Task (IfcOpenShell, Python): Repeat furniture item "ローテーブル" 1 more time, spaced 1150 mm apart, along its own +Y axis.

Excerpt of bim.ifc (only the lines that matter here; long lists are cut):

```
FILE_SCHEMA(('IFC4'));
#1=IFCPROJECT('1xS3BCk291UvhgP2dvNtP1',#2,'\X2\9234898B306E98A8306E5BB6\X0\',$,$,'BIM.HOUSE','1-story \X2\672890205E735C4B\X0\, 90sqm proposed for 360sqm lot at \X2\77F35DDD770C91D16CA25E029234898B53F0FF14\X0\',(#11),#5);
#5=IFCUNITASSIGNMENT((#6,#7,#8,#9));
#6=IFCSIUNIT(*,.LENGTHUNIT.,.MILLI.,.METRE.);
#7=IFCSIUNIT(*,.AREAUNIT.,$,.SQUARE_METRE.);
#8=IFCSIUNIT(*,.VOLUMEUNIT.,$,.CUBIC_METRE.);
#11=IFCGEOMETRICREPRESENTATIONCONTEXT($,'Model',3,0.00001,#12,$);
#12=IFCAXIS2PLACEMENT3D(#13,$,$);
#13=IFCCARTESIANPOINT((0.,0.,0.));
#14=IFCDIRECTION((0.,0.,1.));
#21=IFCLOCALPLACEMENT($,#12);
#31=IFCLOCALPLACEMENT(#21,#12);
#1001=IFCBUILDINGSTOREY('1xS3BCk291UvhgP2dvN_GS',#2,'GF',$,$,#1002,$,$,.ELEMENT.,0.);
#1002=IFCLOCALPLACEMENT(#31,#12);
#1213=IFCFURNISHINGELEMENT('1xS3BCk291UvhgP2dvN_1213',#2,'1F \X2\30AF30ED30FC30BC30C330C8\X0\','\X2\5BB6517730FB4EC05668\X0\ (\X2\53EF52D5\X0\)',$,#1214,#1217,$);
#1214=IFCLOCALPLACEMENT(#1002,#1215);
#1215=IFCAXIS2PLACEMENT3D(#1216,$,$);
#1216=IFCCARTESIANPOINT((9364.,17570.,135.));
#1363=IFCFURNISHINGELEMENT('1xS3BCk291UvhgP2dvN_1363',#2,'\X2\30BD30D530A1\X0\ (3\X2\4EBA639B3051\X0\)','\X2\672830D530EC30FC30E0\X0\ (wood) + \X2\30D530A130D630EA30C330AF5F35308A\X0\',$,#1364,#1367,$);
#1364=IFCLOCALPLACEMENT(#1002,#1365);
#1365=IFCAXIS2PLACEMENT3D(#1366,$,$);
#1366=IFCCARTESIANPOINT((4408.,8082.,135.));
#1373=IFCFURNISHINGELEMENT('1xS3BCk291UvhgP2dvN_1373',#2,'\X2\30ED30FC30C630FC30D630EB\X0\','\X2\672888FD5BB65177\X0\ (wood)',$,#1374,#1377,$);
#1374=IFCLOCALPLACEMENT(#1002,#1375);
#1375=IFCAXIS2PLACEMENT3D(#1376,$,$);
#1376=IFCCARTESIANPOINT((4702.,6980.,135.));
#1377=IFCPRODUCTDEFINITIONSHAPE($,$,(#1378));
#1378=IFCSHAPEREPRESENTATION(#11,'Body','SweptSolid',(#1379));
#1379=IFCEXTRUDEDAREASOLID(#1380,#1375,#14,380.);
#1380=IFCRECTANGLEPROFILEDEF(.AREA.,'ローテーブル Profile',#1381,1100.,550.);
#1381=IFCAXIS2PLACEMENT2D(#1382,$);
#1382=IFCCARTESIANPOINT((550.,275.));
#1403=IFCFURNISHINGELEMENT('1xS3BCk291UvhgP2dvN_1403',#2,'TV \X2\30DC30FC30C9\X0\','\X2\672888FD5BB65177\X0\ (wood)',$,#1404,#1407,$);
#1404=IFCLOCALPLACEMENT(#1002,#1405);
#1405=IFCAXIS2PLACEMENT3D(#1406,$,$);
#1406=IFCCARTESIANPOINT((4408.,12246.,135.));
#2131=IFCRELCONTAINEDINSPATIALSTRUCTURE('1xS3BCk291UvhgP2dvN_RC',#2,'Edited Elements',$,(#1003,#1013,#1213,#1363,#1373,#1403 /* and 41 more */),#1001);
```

```python
import ifcopenshell
import ifcopenshell.api.geometry
import ifcopenshell.api.root
import ifcopenshell.util.element
import ifcopenshell.util.placement

model = ifcopenshell.open("bim.ifc")


def reuse_history(source, copy):
    """copy_class also copies each property set's owner history, people and application; keep the originals."""
    for rel in copy.IsDefinedBy:
        if rel.is_a("IfcRelDefinesByProperties") and (history := rel.RelatingPropertyDefinition.OwnerHistory):
            rel.RelatingPropertyDefinition.OwnerHistory = source.OwnerHistory
            ifcopenshell.util.element.remove_deep2(model, history)


source = model.by_id(1373)
base = ifcopenshell.util.placement.get_local_placement(source.ObjectPlacement)
step = base[:3, 1] * 1150.0

for i in range(1, 2):
    copy = ifcopenshell.api.root.copy_class(model, product=source)
    copy.Representation = ifcopenshell.util.element.copy_deep(
        model, source.Representation, exclude=["IfcGeometricRepresentationContext", "IfcRepresentationMap"]
    )
    reuse_history(source, copy)
    matrix = base.copy()
    matrix[:3, 3] += i * step
    print("added at", matrix[:3, 3].round(3) + 0.0)
    ifcopenshell.api.geometry.edit_object_placement(model, product=copy, matrix=matrix, is_si=False)

model.write("bim-out.ifc")
```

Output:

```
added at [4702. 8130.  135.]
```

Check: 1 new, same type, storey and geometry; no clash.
